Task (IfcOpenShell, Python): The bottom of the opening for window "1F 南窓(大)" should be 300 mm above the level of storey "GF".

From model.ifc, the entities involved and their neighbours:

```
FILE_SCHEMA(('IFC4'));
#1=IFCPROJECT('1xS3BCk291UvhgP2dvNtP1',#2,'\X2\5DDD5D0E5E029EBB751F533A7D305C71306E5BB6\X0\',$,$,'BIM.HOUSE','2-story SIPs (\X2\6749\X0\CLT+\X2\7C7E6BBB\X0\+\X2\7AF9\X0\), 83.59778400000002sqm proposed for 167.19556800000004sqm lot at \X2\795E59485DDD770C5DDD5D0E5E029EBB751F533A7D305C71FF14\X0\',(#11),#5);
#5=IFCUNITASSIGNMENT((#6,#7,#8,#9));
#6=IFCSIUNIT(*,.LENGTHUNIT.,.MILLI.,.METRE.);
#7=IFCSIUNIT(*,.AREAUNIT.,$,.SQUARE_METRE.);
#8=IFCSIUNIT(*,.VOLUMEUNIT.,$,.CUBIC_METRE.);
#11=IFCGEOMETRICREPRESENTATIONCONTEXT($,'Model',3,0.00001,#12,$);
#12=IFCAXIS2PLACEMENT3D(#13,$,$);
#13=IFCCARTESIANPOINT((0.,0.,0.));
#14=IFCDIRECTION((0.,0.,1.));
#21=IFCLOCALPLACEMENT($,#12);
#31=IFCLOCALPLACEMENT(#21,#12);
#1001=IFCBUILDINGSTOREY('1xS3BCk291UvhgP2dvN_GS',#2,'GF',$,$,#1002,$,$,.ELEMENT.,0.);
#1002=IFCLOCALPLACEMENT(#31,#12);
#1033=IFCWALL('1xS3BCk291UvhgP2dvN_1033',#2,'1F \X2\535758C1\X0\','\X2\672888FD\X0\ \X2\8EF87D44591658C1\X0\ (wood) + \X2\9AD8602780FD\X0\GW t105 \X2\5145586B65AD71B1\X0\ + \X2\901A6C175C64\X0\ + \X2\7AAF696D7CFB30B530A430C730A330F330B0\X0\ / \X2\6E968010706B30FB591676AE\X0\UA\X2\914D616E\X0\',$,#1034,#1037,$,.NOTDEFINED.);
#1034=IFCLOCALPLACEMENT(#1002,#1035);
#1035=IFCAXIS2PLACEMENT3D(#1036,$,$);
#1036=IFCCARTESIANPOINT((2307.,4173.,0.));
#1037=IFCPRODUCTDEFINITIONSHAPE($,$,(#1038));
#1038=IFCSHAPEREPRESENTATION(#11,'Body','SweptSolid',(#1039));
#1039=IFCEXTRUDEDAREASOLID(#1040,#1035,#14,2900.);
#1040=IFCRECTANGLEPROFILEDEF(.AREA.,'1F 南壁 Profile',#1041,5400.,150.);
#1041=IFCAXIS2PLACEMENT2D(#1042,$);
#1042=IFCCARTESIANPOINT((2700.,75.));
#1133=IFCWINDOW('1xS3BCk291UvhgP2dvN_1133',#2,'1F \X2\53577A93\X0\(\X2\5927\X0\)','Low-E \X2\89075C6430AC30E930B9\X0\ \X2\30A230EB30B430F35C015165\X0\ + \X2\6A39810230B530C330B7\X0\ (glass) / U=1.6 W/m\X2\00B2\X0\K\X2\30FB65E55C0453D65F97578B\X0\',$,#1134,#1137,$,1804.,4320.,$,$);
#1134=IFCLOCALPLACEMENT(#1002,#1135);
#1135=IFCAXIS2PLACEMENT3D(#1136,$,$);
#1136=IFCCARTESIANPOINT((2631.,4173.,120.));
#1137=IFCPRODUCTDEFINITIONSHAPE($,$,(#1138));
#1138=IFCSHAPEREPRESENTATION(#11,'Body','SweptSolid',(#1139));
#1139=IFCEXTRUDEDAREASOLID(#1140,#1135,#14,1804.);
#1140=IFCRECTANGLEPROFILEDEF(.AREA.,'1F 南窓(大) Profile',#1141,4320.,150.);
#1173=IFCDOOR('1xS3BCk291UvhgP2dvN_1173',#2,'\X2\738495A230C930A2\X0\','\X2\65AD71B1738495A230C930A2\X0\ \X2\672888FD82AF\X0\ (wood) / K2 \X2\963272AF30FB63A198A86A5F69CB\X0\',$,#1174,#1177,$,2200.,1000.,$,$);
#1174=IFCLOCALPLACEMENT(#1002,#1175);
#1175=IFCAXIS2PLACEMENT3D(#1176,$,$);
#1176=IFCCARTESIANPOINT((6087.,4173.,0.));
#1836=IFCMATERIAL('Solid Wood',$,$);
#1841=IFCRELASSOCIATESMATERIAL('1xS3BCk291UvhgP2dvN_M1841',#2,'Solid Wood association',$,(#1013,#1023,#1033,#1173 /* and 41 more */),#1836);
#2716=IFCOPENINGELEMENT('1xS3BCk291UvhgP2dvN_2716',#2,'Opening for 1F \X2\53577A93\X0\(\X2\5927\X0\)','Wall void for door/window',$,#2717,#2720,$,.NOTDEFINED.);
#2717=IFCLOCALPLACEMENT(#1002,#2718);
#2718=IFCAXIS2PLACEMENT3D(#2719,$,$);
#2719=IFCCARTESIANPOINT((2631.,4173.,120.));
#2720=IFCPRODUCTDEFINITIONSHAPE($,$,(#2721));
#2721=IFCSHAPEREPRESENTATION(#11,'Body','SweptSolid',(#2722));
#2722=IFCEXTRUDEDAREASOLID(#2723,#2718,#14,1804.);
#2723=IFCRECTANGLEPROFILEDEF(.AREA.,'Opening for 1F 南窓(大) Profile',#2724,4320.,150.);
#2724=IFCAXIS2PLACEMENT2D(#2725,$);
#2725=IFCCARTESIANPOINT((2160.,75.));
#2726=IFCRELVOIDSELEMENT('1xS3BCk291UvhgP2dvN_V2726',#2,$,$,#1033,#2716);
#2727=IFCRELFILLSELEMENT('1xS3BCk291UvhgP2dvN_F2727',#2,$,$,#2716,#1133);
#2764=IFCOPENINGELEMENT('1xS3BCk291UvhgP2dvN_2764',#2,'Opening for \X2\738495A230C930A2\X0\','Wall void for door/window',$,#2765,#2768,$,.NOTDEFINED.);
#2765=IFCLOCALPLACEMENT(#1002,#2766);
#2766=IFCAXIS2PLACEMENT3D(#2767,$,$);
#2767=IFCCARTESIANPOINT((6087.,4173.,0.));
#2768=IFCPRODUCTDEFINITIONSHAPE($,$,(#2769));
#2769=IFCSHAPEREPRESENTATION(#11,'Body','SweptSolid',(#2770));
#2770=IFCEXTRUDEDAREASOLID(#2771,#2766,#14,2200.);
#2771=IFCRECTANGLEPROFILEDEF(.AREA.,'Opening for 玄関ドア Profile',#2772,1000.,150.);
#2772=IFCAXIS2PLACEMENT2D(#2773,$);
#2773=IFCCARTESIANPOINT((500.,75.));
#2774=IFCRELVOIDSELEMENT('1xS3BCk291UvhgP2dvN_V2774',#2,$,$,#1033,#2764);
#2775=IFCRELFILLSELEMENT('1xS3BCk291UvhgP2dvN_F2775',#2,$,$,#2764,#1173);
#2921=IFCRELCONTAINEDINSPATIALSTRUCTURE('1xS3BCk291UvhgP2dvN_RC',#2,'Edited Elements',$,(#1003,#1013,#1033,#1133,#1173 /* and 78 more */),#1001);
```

```python
import numpy as np
import ifcopenshell
import ifcopenshell.api.geometry
import ifcopenshell.geom
import ifcopenshell.util.element
import ifcopenshell.util.placement
import ifcopenshell.util.shape
import ifcopenshell.util.unit

model = ifcopenshell.open("model.ifc")
unit_scale = ifcopenshell.util.unit.calculate_unit_scale(model)

window = model.by_guid("1xS3BCk291UvhgP2dvN_1133")
opening = window.FillsVoids[0].RelatingOpeningElement
storey = ifcopenshell.util.element.get_container(window, ifc_class="IfcBuildingStorey")
level = ifcopenshell.util.placement.get_local_placement(storey.ObjectPlacement)[2, 3]

# The opening's origin need not be at the sill, so measure its lowest point.
shape = ifcopenshell.geom.create_shape(ifcopenshell.geom.settings(), opening)
bottom = ifcopenshell.util.shape.get_shape_bottom_elevation(shape, shape.geometry) / unit_scale
dz = level + 300.0 - bottom

shift = np.array([0.0, 0.0, dz])
# The window is not placed relative to its opening, so move both.
for product in (opening, window):
    matrix = ifcopenshell.util.placement.get_local_placement(product.ObjectPlacement)
    matrix[:3, 3] += shift
    ifcopenshell.api.geometry.edit_object_placement(model, product=product, matrix=matrix, is_si=False)

print(f"moved by {dz * unit_scale:+.3f} m")

model.write("model_rev.ifc")
```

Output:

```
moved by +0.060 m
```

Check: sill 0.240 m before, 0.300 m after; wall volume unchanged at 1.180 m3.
